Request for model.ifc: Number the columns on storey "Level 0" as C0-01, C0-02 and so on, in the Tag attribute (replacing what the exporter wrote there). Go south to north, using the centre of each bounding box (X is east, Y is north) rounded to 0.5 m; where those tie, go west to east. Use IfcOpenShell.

First a look at what the model holds.

```python
import ifcopenshell
import ifcopenshell.util.element
import ifcopenshell.util.placement

model = ifcopenshell.open("model.ifc")
print(model.schema)
storey = next(s for s in model.by_type("IfcBuildingStorey") if s.Name == "Level 0")
columns = [e for e in ifcopenshell.util.element.get_decomposition(storey) if e.is_a("IfcColumn")]
for e in sorted(columns, key=lambda e: e.id()):
    origin = ifcopenshell.util.placement.get_local_placement(e.ObjectPlacement)[:3, 3]
    print(e.id(), e.Tag, e.Name, origin.round(2) + 0.0, sep=" | ")
```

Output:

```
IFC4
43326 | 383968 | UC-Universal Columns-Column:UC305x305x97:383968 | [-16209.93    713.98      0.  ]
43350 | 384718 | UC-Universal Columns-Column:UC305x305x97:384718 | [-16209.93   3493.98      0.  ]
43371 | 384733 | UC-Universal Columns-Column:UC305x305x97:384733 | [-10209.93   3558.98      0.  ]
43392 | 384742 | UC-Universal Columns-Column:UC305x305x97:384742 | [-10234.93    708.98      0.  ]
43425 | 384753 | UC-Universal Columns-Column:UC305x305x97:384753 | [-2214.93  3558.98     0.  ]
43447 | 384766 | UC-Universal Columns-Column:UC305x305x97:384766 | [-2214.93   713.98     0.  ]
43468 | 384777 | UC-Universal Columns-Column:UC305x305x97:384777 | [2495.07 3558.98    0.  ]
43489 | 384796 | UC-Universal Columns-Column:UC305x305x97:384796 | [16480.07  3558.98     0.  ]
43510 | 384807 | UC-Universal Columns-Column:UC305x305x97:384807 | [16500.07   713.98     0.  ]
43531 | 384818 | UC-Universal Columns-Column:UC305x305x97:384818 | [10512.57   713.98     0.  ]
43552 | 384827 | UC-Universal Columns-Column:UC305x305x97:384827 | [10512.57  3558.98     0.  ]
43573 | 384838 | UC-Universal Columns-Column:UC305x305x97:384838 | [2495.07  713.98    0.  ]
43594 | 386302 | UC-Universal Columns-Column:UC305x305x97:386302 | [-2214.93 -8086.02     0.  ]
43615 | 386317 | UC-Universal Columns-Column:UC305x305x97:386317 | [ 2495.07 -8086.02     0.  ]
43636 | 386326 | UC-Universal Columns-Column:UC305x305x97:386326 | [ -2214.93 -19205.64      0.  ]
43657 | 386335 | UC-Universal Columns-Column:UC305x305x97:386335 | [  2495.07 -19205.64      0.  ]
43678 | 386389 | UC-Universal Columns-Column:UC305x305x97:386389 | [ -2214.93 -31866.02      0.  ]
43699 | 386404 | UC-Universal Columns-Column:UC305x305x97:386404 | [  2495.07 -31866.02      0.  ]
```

```python
import ifcopenshell
import ifcopenshell.geom
import ifcopenshell.util.element
import ifcopenshell.util.shape

model = ifcopenshell.open("model.ifc")
settings = ifcopenshell.geom.settings()
settings.set("use-world-coords", True)


def centre(element):
    shape = ifcopenshell.geom.create_shape(settings, element)
    return ifcopenshell.util.shape.get_bbox_centroid(shape.geometry)


storey = next(s for s in model.by_type("IfcBuildingStorey") if s.Name == "Level 0")
columns = [e for e in ifcopenshell.util.element.get_decomposition(storey) if e.is_a("IfcColumn")]

# Insertion points can sit at a corner or the storey origin, so sort by the geometry (in metres).
centres = {e: centre(e) for e in columns}
columns.sort(key=lambda e: (round(centres[e][1] / 0.5), centres[e][0]))

for i, e in enumerate(columns, start=1):
    number = f"C0-{i:02d}"
    e.Tag = number
    print(e.id(), number)

model.write("model_v2.ifc")
```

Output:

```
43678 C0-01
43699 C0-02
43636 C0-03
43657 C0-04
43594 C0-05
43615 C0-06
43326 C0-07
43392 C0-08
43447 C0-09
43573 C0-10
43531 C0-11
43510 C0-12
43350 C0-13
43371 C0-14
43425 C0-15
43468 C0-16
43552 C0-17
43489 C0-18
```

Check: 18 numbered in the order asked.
